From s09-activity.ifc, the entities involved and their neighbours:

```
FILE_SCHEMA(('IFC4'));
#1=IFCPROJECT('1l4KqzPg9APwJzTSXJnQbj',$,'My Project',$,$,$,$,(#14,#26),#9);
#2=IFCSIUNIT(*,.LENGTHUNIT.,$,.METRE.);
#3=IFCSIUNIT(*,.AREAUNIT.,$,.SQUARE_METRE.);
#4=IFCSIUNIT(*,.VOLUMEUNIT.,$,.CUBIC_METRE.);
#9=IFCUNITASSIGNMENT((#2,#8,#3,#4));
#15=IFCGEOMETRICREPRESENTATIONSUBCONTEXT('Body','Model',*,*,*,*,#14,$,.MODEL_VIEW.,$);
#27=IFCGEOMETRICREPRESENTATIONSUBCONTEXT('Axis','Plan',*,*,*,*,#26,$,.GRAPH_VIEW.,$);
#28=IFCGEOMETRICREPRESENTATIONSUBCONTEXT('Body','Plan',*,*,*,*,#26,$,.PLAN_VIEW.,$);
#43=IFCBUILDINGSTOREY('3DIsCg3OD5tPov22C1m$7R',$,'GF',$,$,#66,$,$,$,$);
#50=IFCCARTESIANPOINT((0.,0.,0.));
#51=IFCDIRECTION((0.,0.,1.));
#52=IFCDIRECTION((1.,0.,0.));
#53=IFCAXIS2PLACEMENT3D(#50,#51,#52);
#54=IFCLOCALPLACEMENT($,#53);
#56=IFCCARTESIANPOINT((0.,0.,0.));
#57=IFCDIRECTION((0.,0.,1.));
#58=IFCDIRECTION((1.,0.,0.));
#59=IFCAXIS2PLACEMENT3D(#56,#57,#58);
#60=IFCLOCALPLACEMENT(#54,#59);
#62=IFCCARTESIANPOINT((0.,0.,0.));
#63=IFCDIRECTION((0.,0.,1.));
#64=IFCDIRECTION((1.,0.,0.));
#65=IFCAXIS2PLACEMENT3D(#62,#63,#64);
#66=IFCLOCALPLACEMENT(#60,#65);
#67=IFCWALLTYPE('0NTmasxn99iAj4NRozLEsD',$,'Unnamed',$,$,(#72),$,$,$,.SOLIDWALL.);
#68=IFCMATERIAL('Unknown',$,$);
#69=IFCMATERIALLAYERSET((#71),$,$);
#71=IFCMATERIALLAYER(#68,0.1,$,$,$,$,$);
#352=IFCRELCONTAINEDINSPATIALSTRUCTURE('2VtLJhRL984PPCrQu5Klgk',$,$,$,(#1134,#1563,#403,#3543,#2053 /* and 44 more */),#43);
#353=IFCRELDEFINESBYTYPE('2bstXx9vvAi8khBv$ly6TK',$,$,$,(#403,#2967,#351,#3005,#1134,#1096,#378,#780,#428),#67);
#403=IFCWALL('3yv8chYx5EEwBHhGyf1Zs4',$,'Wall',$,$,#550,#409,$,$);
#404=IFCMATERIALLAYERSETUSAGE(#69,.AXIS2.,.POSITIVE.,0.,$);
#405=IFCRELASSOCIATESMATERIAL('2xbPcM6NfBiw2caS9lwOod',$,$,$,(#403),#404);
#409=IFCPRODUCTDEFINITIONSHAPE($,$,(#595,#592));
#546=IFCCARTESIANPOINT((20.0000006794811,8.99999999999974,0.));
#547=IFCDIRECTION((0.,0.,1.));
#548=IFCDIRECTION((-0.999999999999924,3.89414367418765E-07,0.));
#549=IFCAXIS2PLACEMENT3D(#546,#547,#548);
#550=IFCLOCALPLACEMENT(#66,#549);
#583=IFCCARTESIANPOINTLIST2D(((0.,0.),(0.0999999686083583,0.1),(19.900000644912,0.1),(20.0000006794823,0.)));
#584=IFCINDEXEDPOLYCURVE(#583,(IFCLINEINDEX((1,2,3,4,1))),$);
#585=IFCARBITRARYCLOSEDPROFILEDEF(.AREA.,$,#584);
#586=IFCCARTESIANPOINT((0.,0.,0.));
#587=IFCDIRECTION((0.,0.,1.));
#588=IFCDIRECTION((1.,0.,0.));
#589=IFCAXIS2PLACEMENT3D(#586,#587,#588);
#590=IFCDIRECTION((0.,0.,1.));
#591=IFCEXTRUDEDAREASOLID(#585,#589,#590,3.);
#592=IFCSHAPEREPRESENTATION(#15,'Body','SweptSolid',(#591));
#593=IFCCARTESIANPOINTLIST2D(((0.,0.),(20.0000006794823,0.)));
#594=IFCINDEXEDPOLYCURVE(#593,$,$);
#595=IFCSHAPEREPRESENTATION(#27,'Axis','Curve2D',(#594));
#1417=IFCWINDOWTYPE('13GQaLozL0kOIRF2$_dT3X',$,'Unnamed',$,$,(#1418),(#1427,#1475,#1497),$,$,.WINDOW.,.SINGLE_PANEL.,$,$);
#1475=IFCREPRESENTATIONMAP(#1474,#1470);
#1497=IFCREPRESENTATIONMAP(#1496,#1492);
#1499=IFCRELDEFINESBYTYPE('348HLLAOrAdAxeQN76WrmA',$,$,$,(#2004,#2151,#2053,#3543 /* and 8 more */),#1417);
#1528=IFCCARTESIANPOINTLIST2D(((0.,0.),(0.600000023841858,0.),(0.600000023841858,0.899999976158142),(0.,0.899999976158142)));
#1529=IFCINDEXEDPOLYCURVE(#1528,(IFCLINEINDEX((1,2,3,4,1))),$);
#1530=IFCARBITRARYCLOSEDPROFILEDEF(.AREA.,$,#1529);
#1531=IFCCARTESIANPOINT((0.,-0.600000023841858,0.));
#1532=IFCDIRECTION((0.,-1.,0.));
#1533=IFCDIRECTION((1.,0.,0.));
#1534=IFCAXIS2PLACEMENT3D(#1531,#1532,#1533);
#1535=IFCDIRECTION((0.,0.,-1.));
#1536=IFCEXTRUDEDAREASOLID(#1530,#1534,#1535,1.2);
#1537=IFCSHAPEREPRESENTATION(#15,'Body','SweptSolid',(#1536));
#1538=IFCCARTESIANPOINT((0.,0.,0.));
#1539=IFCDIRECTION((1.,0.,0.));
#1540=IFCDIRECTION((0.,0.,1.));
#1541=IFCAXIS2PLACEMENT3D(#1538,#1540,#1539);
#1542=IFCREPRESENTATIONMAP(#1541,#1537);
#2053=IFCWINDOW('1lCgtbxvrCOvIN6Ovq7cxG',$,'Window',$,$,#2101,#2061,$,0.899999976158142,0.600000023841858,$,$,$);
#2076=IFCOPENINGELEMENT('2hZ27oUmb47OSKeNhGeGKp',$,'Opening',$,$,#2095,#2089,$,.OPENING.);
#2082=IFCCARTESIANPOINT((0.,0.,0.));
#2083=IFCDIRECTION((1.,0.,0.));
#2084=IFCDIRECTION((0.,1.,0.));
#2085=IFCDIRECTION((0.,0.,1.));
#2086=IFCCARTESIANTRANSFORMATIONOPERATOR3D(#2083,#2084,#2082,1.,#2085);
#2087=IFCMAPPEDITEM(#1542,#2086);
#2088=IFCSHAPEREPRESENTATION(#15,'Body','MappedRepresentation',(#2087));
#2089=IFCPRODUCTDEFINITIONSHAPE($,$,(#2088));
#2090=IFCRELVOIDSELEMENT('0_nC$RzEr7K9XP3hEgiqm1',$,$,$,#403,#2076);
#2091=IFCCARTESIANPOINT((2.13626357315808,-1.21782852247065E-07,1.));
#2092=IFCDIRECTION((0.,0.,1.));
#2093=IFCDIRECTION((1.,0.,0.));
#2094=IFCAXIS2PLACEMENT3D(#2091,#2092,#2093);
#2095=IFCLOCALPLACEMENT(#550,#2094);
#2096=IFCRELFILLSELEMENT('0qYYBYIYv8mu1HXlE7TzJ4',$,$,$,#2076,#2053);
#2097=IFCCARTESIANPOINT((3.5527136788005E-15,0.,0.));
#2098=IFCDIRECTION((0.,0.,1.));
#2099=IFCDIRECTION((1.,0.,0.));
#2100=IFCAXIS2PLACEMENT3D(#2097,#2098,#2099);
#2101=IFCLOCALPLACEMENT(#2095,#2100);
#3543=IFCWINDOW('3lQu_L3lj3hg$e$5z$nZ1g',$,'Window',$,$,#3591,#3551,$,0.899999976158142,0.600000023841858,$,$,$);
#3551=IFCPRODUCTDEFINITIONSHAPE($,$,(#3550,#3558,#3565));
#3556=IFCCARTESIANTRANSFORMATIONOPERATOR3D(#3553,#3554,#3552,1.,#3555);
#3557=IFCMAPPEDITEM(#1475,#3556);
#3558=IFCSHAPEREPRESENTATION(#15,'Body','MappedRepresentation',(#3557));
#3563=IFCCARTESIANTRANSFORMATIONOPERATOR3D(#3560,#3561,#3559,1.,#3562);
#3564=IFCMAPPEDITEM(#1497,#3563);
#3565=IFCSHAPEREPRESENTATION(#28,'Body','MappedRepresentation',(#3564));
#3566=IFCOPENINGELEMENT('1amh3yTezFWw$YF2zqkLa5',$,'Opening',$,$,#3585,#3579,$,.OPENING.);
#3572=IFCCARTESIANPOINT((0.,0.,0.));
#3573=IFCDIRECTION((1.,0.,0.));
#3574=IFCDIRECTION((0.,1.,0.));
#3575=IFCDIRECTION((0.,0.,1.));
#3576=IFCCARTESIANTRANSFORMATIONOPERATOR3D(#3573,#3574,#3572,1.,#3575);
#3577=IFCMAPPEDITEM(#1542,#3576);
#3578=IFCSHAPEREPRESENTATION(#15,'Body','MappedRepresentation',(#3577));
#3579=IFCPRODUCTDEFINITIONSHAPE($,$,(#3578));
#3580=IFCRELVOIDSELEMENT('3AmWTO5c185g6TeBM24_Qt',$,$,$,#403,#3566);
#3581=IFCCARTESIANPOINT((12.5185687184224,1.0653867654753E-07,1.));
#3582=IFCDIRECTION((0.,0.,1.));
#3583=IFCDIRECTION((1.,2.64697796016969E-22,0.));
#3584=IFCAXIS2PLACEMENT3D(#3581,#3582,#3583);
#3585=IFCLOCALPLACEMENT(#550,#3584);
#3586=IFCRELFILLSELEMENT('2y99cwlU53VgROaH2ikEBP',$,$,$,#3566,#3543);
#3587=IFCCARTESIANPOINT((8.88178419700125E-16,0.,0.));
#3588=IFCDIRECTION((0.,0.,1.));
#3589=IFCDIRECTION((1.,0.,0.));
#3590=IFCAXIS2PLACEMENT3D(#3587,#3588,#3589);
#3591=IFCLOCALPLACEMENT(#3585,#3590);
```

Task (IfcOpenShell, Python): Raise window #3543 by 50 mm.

```python
import numpy as np
import ifcopenshell
import ifcopenshell.api.geometry
import ifcopenshell.util.placement
import ifcopenshell.util.unit

model = ifcopenshell.open("s09-activity.ifc")
unit_scale = ifcopenshell.util.unit.calculate_unit_scale(model)

window = model.by_guid("3lQu_L3lj3hg$e$5z$nZ1g")
opening = window.FillsVoids[0].RelatingOpeningElement
dz = 0.05 / unit_scale

shift = np.array([0.0, 0.0, dz])
# The window is placed relative to its opening, so it follows when the opening moves.
matrix = ifcopenshell.util.placement.get_local_placement(opening.ObjectPlacement)
matrix[:3, 3] += shift
ifcopenshell.api.geometry.edit_object_placement(
    model, product=opening, matrix=matrix, is_si=False, should_transform_children=True
)

print(f"moved by {dz * unit_scale:+.3f} m")

model.write("s09-activity_v2.ifc")
```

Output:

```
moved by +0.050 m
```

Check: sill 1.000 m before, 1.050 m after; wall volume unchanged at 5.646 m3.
